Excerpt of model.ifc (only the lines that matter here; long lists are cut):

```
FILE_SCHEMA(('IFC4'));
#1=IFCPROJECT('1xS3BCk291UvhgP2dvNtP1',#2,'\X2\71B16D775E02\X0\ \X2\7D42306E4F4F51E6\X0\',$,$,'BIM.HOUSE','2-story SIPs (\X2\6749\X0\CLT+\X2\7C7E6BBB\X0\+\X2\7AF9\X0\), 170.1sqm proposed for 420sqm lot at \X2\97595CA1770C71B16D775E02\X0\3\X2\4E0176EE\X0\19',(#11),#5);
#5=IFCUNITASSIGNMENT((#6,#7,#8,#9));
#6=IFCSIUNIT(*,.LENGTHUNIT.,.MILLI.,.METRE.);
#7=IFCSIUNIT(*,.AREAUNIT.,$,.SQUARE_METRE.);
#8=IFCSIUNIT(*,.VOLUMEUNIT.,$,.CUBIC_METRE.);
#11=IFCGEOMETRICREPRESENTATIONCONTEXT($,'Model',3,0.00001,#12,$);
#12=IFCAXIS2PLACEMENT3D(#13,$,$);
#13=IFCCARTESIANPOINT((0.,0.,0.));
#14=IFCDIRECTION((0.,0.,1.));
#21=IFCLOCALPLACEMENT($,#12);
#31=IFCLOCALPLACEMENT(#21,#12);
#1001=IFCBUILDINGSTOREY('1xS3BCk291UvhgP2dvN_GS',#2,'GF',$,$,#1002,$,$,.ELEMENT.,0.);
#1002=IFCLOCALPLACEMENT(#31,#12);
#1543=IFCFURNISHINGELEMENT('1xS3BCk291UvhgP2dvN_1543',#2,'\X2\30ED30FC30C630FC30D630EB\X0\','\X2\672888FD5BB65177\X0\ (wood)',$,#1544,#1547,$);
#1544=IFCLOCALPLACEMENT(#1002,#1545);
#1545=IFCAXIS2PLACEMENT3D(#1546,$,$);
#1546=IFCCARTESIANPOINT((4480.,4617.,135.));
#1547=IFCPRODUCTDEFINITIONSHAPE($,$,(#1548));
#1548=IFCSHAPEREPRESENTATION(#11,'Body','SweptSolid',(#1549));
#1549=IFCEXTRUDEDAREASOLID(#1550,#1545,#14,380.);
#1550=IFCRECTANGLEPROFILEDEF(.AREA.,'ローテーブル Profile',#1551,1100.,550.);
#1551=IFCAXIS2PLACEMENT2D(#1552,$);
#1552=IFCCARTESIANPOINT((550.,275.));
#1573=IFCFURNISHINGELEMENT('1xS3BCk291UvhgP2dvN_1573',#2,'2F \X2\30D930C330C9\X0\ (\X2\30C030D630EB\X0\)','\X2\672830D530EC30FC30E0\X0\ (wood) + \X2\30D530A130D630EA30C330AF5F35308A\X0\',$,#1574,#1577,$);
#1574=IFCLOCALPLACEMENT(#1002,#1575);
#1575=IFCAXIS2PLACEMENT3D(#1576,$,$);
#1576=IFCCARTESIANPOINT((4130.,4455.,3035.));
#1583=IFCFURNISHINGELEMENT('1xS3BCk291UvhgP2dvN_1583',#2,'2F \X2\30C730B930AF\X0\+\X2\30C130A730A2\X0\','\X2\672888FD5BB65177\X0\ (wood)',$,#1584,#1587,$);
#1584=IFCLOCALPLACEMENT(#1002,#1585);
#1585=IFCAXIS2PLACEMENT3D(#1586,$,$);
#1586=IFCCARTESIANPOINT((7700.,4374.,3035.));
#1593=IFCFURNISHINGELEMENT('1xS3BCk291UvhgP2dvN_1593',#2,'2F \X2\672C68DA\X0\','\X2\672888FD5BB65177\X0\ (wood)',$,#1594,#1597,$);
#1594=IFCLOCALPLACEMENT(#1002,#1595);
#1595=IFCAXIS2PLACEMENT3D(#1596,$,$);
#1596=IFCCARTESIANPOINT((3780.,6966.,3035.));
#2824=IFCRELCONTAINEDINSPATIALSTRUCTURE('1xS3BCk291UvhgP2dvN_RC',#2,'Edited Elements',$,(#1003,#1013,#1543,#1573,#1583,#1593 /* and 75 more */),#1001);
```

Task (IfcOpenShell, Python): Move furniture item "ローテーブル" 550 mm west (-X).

```python
import ifcopenshell
import ifcopenshell.api.geometry
import ifcopenshell.util.placement
import ifcopenshell.util.unit

model = ifcopenshell.open("model.ifc")
unit_scale = ifcopenshell.util.unit.calculate_unit_scale(model)

item = model.by_guid("1xS3BCk291UvhgP2dvN_1543")
matrix = ifcopenshell.util.placement.get_local_placement(item.ObjectPlacement)
matrix[0, 3] -= 0.55 / unit_scale
ifcopenshell.api.geometry.edit_object_placement(model, product=item, matrix=matrix, is_si=False)

print(ifcopenshell.util.placement.get_local_placement(item.ObjectPlacement).round(3) + 0.0)

model.write("model_edited.ifc")
```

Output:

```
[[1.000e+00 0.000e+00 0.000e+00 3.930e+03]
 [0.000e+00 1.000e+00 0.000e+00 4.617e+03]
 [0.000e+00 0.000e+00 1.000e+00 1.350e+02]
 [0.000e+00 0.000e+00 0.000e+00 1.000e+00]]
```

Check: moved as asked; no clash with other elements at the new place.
